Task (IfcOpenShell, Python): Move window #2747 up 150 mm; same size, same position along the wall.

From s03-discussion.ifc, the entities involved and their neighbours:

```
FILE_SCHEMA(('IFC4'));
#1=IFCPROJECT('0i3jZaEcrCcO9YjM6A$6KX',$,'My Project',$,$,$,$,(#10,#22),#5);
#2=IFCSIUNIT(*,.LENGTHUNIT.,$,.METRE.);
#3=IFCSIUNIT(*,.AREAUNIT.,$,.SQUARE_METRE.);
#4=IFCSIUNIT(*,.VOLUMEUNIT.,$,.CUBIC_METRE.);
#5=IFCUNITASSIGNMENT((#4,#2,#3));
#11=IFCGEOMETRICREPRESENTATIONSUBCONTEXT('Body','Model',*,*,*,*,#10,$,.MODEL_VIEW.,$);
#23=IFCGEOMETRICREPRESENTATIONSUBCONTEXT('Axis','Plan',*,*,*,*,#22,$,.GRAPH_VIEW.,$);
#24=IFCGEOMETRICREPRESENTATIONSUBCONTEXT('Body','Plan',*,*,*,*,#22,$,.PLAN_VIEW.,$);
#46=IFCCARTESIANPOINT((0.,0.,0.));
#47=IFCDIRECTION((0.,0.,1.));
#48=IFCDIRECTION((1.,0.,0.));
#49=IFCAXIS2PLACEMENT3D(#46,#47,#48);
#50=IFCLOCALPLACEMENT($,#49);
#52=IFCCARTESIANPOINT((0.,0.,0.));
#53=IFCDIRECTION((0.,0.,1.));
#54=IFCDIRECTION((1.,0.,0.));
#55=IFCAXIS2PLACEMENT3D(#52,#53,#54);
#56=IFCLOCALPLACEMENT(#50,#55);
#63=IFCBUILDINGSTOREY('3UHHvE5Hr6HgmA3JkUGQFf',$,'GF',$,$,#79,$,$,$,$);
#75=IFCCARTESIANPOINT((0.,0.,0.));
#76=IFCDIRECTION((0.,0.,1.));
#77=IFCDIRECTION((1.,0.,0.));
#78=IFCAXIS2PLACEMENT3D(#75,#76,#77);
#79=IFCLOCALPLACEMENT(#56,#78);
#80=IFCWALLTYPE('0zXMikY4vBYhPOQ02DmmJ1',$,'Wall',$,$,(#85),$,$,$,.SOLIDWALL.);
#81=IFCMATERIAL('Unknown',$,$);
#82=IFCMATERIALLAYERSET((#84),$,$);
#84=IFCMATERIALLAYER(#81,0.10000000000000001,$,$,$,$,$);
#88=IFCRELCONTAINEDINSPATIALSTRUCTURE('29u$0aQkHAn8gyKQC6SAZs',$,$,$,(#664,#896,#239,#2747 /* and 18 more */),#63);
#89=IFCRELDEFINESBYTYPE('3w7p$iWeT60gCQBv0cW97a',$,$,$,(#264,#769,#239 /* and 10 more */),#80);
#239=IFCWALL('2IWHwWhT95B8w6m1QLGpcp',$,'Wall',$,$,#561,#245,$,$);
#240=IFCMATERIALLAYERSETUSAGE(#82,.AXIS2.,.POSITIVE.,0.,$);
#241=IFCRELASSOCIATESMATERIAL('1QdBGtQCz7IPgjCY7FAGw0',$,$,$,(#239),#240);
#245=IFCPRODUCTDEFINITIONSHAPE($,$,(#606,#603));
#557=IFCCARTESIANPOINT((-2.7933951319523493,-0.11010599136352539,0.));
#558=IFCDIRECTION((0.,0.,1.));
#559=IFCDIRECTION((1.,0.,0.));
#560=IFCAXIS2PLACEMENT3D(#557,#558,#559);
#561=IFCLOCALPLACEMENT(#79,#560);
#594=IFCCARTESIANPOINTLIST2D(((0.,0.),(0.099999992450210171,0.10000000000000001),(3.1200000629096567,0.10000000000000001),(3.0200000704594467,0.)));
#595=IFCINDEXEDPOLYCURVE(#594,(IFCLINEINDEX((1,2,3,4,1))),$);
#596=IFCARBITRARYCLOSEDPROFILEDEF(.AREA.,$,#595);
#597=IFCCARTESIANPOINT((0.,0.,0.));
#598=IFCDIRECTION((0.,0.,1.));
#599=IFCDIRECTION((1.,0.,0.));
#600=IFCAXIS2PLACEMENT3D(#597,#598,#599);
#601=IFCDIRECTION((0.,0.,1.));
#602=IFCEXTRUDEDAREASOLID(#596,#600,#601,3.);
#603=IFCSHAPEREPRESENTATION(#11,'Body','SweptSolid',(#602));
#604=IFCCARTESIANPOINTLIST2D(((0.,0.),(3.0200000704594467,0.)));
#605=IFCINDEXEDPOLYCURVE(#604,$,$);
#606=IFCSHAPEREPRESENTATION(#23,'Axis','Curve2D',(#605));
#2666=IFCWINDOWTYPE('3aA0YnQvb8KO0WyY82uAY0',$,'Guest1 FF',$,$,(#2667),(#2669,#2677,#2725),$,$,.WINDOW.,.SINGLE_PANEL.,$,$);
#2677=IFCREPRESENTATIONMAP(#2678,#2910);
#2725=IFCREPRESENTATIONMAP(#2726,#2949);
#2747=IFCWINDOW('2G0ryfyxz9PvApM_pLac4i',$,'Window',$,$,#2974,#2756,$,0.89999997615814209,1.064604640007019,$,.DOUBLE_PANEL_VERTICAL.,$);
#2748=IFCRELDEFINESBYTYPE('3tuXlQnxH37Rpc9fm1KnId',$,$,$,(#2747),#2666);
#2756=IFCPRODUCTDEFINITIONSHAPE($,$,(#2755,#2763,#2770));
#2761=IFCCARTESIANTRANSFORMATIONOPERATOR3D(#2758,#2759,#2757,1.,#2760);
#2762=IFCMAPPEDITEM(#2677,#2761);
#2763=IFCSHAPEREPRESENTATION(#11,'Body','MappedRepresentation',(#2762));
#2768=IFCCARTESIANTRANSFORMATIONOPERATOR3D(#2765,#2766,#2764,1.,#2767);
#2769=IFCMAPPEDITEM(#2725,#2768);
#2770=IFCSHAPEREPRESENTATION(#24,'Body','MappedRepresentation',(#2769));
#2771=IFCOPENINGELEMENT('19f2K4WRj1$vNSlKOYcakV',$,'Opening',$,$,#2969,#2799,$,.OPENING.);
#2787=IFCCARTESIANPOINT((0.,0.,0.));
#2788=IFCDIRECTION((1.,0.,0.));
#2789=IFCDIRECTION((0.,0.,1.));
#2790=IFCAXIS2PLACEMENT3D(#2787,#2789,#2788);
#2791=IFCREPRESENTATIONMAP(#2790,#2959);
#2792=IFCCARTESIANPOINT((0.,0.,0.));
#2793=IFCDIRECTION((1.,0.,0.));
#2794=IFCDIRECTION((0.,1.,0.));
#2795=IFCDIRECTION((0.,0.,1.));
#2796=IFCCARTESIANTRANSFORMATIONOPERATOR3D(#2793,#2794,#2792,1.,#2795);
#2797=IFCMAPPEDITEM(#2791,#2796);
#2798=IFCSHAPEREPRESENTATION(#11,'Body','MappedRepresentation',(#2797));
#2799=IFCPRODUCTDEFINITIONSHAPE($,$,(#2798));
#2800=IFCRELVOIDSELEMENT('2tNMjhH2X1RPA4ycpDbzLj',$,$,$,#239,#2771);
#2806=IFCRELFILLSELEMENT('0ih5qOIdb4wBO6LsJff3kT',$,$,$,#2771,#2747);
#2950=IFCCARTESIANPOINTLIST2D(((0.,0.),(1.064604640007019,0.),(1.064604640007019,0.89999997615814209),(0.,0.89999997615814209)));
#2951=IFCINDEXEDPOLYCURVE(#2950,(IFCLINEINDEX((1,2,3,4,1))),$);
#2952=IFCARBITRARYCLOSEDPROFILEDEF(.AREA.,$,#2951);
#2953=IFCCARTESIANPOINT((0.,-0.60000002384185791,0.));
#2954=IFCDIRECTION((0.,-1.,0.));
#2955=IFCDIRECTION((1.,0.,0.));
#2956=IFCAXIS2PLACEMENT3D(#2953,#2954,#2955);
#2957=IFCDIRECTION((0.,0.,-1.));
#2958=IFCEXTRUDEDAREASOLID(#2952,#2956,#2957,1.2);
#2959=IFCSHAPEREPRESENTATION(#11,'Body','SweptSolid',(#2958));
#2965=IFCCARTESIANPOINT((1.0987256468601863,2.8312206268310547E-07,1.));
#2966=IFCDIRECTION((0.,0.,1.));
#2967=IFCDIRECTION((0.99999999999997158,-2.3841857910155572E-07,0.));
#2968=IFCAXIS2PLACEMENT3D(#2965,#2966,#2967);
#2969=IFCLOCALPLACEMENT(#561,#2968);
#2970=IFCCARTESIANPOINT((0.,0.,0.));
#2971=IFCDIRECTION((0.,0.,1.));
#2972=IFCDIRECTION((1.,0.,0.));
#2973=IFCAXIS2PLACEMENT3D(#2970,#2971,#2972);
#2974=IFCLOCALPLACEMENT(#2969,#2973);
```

```python
import numpy as np
import ifcopenshell
import ifcopenshell.api.geometry
import ifcopenshell.util.placement
import ifcopenshell.util.unit

model = ifcopenshell.open("s03-discussion.ifc")
unit_scale = ifcopenshell.util.unit.calculate_unit_scale(model)

window = model.by_guid("2G0ryfyxz9PvApM_pLac4i")
opening = window.FillsVoids[0].RelatingOpeningElement
dz = 0.15

shift = np.array([0.0, 0.0, dz])
# The window is placed relative to its opening, so it follows when the opening moves.
matrix = ifcopenshell.util.placement.get_local_placement(opening.ObjectPlacement)
matrix[:3, 3] += shift
ifcopenshell.api.geometry.edit_object_placement(
    model, product=opening, matrix=matrix, is_si=False, should_transform_children=True
)

print(f"moved by {dz * unit_scale:+.3f} m")

model.write("s03-discussion_updated.ifc")
```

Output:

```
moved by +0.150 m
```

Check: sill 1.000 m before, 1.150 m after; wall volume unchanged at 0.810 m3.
